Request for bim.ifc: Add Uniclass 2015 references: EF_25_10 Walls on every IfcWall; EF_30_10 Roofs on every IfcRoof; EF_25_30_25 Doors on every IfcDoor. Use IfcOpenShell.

First a look at what the model holds.

```python
import ifcopenshell

model = ifcopenshell.open("bim.ifc")
print(model.schema)
print("classifications:", [c.Name for c in model.by_type("IfcClassification")])
for ifc_class in ("IfcDoor", "IfcRoof", "IfcStair", "IfcWall", "IfcWindow"):
    print(ifc_class, len(model.by_type(ifc_class)))
```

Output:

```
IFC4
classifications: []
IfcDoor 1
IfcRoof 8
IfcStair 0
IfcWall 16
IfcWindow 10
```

```python
import ifcopenshell
import ifcopenshell.api.classification

model = ifcopenshell.open("bim.ifc")

system = ifcopenshell.api.classification.add_classification(model, classification="Uniclass 2015")

codes = {
    "IfcWall": ("EF_25_10", "Walls"),
    "IfcRoof": ("EF_30_10", "Roofs"),
    "IfcDoor": ("EF_25_30_25", "Doors"),
}
for ifc_class, (code, name) in codes.items():
    products = model.by_type(ifc_class)
    ifcopenshell.api.classification.add_reference(
        model, products=products, classification=system, identification=code, name=name
    )
    print(code, len(products))

model.write("bim_v2.ifc")
```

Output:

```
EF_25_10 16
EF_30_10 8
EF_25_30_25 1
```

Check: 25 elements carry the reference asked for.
